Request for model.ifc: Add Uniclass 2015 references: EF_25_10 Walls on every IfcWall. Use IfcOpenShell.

First a look at what the model holds.

```python
import ifcopenshell

model = ifcopenshell.open("model.ifc")
print(model.schema)
print("classifications:", [c.Name for c in model.by_type("IfcClassification")])
for ifc_class in ("IfcDoor", "IfcRoof", "IfcStair", "IfcWall", "IfcWindow"):
    print(ifc_class, len(model.by_type(ifc_class)))
```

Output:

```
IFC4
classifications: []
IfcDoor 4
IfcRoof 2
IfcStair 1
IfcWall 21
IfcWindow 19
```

```python
import ifcopenshell
import ifcopenshell.api.classification

model = ifcopenshell.open("model.ifc")

system = ifcopenshell.api.classification.add_classification(model, classification="Uniclass 2015")

codes = {
    "IfcWall": ("EF_25_10", "Walls"),
}
for ifc_class, (code, name) in codes.items():
    products = model.by_type(ifc_class)
    ifcopenshell.api.classification.add_reference(
        model, products=products, classification=system, identification=code, name=name
    )
    print(code, len(products))

model.write("model-out.ifc")
```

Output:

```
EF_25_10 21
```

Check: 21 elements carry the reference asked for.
